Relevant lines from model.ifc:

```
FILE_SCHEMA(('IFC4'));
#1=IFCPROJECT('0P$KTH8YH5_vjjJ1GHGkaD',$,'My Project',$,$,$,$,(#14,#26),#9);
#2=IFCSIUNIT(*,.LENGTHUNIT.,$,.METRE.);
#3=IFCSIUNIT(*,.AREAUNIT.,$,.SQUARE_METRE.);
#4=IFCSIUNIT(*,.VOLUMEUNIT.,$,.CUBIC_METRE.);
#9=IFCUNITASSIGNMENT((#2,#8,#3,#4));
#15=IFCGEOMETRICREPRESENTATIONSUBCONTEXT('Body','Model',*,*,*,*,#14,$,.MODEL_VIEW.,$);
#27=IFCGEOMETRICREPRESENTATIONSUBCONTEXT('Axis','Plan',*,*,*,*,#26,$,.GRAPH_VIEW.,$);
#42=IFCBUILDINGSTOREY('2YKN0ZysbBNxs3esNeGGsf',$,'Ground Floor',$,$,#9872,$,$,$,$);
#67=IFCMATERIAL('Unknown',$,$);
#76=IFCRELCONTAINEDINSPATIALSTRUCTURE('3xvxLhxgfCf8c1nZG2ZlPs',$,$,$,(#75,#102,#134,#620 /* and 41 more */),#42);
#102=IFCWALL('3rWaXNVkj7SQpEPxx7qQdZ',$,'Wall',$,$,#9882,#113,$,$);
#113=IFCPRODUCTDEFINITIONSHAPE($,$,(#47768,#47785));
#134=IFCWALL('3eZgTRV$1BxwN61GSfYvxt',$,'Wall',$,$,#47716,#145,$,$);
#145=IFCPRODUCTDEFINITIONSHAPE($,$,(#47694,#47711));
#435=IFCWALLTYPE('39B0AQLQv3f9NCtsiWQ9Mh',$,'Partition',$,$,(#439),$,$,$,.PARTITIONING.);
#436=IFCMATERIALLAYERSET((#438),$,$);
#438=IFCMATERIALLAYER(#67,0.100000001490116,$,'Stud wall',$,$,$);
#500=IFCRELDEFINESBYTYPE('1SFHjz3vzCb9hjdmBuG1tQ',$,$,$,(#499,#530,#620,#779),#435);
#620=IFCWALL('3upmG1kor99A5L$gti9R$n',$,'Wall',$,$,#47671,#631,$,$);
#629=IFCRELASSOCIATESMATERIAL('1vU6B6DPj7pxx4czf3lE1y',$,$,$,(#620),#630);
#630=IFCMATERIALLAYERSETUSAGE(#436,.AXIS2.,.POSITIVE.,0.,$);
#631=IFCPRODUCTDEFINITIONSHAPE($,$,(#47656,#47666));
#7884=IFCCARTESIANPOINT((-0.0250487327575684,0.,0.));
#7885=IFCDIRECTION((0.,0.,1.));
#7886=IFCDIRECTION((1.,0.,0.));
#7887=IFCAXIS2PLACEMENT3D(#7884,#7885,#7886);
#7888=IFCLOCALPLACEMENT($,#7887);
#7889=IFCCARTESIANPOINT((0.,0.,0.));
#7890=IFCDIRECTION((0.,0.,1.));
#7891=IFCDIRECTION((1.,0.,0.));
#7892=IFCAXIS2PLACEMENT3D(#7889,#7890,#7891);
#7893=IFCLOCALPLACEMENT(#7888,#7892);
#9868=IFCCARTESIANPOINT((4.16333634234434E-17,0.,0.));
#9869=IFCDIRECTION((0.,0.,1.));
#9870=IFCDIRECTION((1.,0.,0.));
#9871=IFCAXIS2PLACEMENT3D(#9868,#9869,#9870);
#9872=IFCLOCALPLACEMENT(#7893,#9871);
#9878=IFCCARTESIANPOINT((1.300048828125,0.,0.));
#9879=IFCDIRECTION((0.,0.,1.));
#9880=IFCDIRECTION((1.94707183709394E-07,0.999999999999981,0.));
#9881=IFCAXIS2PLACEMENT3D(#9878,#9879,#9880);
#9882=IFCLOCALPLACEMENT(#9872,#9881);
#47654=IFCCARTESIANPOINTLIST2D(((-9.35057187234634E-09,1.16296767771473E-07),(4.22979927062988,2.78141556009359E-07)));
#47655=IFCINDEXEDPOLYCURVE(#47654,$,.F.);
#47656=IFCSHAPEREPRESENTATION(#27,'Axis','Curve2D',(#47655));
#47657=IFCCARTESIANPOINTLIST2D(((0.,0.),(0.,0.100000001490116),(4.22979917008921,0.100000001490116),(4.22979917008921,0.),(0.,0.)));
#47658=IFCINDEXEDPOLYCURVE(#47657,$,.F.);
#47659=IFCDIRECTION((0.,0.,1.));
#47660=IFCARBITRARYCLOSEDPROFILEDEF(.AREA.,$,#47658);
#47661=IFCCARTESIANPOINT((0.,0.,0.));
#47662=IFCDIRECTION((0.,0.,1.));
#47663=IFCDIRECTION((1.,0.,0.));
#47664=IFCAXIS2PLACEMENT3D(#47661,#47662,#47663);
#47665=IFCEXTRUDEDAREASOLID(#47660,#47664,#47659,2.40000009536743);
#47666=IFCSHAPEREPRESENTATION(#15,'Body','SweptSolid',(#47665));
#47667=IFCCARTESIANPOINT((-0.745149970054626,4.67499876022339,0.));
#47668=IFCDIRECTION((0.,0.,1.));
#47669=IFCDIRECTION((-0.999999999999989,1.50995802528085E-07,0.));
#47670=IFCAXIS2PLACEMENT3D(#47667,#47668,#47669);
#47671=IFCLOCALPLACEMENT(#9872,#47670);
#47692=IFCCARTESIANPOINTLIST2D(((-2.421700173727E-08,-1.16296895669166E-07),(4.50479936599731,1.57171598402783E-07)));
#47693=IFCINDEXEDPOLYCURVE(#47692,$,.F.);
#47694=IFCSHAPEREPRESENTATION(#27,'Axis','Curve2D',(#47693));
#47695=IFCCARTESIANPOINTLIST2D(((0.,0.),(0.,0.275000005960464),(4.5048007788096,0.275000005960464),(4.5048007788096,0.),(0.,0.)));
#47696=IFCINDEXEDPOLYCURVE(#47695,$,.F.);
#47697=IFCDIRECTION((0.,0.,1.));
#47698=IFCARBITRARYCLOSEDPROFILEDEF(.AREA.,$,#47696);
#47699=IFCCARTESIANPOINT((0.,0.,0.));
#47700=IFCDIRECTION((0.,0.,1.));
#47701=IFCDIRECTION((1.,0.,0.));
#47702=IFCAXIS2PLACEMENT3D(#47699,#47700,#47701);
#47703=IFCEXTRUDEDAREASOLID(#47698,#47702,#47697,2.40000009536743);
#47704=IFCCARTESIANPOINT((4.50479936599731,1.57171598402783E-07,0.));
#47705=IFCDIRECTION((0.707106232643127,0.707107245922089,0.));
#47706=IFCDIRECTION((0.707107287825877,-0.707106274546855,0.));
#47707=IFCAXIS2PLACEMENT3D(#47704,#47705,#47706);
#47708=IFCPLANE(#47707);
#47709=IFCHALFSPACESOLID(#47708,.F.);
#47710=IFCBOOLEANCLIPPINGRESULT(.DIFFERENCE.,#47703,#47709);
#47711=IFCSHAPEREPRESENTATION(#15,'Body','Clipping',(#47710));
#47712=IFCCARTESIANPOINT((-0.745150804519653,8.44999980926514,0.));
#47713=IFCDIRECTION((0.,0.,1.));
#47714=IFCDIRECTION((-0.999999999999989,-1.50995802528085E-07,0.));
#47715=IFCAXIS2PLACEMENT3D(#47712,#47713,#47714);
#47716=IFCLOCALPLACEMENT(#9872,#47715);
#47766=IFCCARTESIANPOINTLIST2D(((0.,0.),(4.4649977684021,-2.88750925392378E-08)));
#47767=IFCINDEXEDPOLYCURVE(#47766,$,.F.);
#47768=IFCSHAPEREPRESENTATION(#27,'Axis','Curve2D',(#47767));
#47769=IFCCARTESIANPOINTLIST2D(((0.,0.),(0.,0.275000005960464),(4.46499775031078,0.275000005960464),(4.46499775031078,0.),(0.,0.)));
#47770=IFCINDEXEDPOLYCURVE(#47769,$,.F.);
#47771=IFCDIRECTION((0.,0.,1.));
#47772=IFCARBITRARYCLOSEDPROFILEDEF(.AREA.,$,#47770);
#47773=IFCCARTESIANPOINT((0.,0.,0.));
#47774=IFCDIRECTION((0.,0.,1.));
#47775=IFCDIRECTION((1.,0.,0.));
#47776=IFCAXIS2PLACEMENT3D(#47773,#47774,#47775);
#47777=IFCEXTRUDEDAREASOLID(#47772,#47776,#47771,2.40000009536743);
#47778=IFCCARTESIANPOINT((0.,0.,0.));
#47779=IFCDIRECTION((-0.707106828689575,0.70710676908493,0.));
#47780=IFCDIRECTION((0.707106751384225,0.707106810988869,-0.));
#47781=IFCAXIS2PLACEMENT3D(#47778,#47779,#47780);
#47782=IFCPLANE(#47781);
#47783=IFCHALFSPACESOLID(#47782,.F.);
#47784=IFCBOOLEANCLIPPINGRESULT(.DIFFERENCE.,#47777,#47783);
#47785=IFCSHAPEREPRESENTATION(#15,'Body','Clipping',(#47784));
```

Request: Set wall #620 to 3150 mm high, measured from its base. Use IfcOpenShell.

```python
import ifcopenshell
import ifcopenshell.geom
import ifcopenshell.util.representation
import ifcopenshell.util.shape
import ifcopenshell.util.unit

model = ifcopenshell.open("model.ifc")
unit_scale = ifcopenshell.util.unit.calculate_unit_scale(model)
settings = ifcopenshell.geom.settings()


def volume(element):
    """Net volume in cubic metres, openings subtracted."""
    shape = ifcopenshell.geom.create_shape(settings, element)
    return ifcopenshell.util.shape.get_volume(shape.geometry)


wall = model.by_id(620)
before = volume(wall)

body = ifcopenshell.util.representation.get_representation(wall, "Model", "Body")
solid = body.Items[0]
old_height = solid.Depth
solid.Depth = 3.15 / unit_scale
after = volume(wall)

print(f"height {old_height:g} -> {solid.Depth:g}, volume {before:.3f} -> {after:.3f} m3")

model.write("model-out.ifc")
```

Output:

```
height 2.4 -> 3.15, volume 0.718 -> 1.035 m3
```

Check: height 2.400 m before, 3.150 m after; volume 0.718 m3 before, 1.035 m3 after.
